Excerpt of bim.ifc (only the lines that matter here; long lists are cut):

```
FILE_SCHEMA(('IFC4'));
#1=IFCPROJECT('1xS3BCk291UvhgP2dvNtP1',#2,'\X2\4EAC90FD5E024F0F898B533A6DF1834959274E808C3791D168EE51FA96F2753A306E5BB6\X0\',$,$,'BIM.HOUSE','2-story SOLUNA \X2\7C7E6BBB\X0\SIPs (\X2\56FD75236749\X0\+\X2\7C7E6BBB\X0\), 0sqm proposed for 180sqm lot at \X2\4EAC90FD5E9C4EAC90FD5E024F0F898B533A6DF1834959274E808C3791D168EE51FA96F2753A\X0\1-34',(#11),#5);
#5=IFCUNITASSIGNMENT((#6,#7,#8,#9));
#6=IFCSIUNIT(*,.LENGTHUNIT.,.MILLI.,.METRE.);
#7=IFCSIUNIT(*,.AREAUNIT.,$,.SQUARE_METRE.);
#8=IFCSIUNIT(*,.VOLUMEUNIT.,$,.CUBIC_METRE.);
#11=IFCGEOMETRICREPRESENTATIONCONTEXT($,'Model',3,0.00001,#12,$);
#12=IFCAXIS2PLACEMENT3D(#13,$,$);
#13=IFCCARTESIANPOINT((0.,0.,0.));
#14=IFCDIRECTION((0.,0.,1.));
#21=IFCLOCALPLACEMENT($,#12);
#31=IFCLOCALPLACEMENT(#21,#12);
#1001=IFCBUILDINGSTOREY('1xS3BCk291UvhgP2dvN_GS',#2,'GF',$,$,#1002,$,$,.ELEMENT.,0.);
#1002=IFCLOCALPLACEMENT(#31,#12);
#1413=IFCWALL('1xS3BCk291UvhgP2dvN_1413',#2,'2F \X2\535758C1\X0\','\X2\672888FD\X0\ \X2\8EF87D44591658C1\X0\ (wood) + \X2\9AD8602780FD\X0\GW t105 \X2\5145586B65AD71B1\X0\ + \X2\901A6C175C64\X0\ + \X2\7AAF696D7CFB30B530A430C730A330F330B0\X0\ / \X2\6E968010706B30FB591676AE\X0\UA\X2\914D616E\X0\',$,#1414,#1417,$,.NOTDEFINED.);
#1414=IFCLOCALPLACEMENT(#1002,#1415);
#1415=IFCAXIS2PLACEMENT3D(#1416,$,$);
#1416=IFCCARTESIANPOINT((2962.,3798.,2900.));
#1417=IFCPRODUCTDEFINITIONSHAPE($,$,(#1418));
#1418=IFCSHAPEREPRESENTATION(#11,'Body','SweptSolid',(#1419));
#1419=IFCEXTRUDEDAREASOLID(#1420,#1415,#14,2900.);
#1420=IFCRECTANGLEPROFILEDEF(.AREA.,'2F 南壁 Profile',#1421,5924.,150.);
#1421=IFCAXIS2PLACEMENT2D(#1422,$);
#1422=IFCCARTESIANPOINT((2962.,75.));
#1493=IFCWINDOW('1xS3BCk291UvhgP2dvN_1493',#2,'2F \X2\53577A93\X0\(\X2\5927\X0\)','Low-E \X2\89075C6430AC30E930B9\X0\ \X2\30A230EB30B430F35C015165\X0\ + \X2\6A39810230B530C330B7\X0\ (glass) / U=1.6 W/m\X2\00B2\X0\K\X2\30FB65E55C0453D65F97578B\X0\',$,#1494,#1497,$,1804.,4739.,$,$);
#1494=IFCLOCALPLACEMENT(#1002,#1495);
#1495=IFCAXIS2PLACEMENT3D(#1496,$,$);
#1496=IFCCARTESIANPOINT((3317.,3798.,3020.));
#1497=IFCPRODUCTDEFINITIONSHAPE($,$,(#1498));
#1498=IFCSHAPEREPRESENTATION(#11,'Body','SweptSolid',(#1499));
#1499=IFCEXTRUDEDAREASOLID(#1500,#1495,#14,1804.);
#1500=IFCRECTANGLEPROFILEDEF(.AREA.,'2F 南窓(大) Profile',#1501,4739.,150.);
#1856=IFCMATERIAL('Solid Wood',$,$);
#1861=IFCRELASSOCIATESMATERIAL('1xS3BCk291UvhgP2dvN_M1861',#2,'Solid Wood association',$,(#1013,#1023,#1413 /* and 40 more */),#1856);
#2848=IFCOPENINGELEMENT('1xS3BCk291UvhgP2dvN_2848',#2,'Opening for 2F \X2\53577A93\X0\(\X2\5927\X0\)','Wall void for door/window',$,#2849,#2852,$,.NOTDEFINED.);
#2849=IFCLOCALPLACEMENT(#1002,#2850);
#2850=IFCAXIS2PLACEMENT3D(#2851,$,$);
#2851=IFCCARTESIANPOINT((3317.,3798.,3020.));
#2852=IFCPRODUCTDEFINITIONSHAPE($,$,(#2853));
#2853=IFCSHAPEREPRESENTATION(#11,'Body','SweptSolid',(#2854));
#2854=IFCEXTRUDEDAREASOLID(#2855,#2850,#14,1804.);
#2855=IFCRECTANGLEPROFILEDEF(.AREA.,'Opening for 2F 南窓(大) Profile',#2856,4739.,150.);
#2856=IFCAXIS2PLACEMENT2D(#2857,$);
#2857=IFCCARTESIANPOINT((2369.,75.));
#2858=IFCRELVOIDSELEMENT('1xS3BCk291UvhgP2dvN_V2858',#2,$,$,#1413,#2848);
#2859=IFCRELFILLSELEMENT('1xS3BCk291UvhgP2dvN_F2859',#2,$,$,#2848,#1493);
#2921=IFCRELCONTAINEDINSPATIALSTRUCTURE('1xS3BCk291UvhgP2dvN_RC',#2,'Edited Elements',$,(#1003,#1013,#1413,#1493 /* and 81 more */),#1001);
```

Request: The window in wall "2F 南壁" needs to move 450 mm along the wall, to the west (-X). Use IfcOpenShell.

```python
import ifcopenshell
import ifcopenshell.api.geometry
import ifcopenshell.util.placement

model = ifcopenshell.open("bim.ifc")

window = model.by_guid("1xS3BCk291UvhgP2dvN_1493")
opening = window.FillsVoids[0].RelatingOpeningElement
wall = opening.VoidsElements[0].RelatingBuildingElement

wall_matrix = ifcopenshell.util.placement.get_local_placement(wall.ObjectPlacement)
shift = wall_matrix[:3, 0] * -450.0
before = ifcopenshell.util.placement.get_local_placement(window.ObjectPlacement)[:3, 3].copy()

# The window is not placed relative to its opening, so move both.
for product in (opening, window):
    matrix = ifcopenshell.util.placement.get_local_placement(product.ObjectPlacement)
    matrix[:3, 3] += shift
    ifcopenshell.api.geometry.edit_object_placement(model, product=product, matrix=matrix, is_si=False)

after = ifcopenshell.util.placement.get_local_placement(window.ObjectPlacement)[:3, 3]
print("window moved by", (after - before).round(3) + 0.0)

model.write("bim_edited.ifc")
```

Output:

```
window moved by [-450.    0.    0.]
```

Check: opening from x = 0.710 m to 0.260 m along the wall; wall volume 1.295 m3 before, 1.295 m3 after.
